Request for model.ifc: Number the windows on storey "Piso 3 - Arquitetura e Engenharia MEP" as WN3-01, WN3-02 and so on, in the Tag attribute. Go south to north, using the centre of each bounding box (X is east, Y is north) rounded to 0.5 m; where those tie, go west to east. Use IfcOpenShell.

First a look at what the model holds.

```python
import ifcopenshell
import ifcopenshell.util.element
import ifcopenshell.util.placement

model = ifcopenshell.open("model.ifc")
print(model.schema)
storey = next(s for s in model.by_type("IfcBuildingStorey") if s.Name == "Piso 3 - Arquitetura e Engenharia MEP")
windows = [e for e in ifcopenshell.util.element.get_decomposition(storey) if e.is_a("IfcWindow")]
for e in sorted(windows, key=lambda e: e.id()):
    origin = ifcopenshell.util.placement.get_local_placement(e.ObjectPlacement)[:3, 3]
    print(e.id(), e.Tag, e.Name, origin.round(2) + 0.0, sep=" | ")
```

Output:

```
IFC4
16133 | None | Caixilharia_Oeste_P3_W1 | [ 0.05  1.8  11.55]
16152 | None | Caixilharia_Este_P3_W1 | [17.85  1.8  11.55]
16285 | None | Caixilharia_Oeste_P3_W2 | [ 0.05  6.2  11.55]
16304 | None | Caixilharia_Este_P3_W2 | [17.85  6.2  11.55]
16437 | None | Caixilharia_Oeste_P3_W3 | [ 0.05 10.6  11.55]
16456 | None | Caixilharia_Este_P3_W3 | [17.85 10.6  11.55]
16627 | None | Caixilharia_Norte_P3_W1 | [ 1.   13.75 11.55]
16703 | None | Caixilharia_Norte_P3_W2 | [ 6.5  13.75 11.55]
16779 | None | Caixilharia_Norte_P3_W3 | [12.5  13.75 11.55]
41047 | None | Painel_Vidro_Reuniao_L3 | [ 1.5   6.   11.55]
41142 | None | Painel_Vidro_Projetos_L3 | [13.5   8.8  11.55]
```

```python
import ifcopenshell
import ifcopenshell.geom
import ifcopenshell.util.element
import ifcopenshell.util.shape

model = ifcopenshell.open("model.ifc")
settings = ifcopenshell.geom.settings()
settings.set("use-world-coords", True)


def centre(element):
    shape = ifcopenshell.geom.create_shape(settings, element)
    return ifcopenshell.util.shape.get_bbox_centroid(shape.geometry)


storey = next(s for s in model.by_type("IfcBuildingStorey") if s.Name == "Piso 3 - Arquitetura e Engenharia MEP")
windows = [e for e in ifcopenshell.util.element.get_decomposition(storey) if e.is_a("IfcWindow")]

# Insertion points can sit at a corner or the storey origin, so sort by the geometry (in metres).
centres = {e: centre(e) for e in windows}
windows.sort(key=lambda e: (round(centres[e][1] / 0.5), centres[e][0]))

for i, e in enumerate(windows, start=1):
    number = f"WN3-{i:02d}"
    e.Tag = number
    print(e.id(), number)

model.write("model-out.ifc")
```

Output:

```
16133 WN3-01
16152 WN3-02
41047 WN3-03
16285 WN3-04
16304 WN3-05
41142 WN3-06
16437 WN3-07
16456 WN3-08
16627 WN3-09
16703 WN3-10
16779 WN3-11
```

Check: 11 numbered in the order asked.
